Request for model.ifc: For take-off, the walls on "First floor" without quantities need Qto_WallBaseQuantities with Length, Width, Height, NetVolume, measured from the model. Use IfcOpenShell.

First a look at what the model holds.

```python
import ifcopenshell
import ifcopenshell.util.element
import ifcopenshell.util.unit

model = ifcopenshell.open("model.ifc")
print(model.schema)
for unit_type in ("LENGTHUNIT", "AREAUNIT", "VOLUMEUNIT"):
    print(unit_type, ifcopenshell.util.unit.calculate_unit_scale(model, unit_type))
storey = next(s for s in model.by_type("IfcBuildingStorey") if s.Name == "First floor")
walls = [e for e in ifcopenshell.util.element.get_decomposition(storey) if e.is_a("IfcWall")]
for e in sorted(walls, key=lambda e: e.id()):
    print(e.id(), e.is_a(), e.Name, list(ifcopenshell.util.element.get_psets(e, qtos_only=True)), sep=" | ")
```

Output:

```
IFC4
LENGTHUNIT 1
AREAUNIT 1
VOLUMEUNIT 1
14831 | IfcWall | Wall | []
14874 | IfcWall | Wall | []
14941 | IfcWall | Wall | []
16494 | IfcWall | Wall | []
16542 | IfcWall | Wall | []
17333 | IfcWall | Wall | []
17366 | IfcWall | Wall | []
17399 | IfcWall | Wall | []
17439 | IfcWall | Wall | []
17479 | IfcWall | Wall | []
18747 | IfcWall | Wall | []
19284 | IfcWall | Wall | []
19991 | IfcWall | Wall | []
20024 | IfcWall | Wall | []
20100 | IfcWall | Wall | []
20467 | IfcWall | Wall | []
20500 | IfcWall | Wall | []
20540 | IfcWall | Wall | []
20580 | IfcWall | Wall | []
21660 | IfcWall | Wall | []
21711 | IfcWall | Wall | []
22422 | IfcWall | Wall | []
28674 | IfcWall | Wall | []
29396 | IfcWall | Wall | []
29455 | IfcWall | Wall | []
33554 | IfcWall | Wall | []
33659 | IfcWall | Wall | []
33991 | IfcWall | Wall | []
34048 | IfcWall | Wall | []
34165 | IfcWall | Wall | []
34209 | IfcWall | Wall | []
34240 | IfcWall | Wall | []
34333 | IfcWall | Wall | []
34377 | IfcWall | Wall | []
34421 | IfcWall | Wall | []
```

```python
import ifcopenshell
import ifcopenshell.api.pset
import ifcopenshell.geom
import ifcopenshell.util.element
import ifcopenshell.util.shape
import ifcopenshell.util.unit

model = ifcopenshell.open("model.ifc")
unit_scale = ifcopenshell.util.unit.calculate_unit_scale(model)
volume_scale = ifcopenshell.util.unit.calculate_unit_scale(model, "VOLUMEUNIT")
settings = ifcopenshell.geom.settings()

storey = next(s for s in model.by_type("IfcBuildingStorey") if s.Name == "First floor")
walls = [e for e in ifcopenshell.util.element.get_decomposition(storey) if e.is_a("IfcWall")]

for e in sorted(walls, key=lambda e: e.id()):
    if ifcopenshell.util.element.get_psets(e, qtos_only=True, should_inherit=False):
        continue
    # Geometry comes back in metres, in the element's own axes.
    shape = ifcopenshell.geom.create_shape(settings, e)
    values = {
        "Length": ifcopenshell.util.shape.get_x(shape.geometry) / unit_scale,
        "Width": ifcopenshell.util.shape.get_y(shape.geometry) / unit_scale,
        "Height": ifcopenshell.util.shape.get_z(shape.geometry) / unit_scale,
        "NetVolume": ifcopenshell.util.shape.get_volume(shape.geometry) / volume_scale,
    }
    qto = ifcopenshell.api.pset.add_qto(model, product=e, name="Qto_WallBaseQuantities")
    ifcopenshell.api.pset.edit_qto(model, qto=qto, properties=values)
    print(e.id(), {k: round(v, 3) for k, v in values.items()})

model.write("model-out.ifc")
```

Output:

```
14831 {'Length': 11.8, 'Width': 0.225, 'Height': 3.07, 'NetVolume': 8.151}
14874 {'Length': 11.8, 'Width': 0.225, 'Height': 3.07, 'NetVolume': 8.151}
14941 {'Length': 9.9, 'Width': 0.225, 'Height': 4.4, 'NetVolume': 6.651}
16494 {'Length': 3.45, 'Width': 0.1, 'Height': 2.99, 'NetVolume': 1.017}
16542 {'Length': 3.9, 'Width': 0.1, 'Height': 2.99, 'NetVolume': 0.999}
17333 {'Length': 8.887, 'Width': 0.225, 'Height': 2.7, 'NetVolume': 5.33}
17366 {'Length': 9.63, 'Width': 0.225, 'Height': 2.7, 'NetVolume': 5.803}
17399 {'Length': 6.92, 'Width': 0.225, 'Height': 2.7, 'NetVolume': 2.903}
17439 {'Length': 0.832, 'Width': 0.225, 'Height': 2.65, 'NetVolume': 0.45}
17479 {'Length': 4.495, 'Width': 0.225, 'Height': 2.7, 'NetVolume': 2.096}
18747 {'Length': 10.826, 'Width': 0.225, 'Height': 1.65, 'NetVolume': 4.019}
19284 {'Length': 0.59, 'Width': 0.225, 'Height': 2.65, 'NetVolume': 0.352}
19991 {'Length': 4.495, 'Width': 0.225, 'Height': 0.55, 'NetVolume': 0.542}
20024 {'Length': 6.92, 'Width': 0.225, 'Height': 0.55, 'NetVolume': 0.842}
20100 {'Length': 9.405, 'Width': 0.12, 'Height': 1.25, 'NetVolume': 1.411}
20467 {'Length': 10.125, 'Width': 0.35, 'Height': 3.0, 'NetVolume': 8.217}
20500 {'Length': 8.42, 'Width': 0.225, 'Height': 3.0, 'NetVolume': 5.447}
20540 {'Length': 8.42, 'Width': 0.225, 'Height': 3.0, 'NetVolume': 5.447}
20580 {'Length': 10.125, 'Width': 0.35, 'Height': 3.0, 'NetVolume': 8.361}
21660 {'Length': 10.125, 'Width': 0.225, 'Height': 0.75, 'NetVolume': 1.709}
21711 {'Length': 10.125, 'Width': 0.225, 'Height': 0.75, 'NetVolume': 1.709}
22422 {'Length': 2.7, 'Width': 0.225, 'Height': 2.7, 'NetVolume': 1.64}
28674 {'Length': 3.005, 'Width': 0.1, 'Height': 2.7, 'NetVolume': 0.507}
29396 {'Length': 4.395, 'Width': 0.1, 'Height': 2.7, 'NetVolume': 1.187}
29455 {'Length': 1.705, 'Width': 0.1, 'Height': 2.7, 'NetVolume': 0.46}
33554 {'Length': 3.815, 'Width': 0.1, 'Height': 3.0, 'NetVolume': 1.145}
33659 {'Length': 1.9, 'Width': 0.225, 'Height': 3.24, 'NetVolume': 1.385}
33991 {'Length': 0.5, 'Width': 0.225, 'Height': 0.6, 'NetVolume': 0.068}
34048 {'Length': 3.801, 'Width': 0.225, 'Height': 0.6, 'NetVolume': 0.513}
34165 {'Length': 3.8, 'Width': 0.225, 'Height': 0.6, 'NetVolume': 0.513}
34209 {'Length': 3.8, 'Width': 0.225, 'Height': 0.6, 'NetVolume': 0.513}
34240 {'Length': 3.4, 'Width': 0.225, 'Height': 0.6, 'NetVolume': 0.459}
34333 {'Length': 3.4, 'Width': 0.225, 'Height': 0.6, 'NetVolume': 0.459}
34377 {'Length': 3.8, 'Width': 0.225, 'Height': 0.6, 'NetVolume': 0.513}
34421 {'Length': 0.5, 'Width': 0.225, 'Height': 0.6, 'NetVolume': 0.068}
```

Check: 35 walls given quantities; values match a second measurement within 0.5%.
